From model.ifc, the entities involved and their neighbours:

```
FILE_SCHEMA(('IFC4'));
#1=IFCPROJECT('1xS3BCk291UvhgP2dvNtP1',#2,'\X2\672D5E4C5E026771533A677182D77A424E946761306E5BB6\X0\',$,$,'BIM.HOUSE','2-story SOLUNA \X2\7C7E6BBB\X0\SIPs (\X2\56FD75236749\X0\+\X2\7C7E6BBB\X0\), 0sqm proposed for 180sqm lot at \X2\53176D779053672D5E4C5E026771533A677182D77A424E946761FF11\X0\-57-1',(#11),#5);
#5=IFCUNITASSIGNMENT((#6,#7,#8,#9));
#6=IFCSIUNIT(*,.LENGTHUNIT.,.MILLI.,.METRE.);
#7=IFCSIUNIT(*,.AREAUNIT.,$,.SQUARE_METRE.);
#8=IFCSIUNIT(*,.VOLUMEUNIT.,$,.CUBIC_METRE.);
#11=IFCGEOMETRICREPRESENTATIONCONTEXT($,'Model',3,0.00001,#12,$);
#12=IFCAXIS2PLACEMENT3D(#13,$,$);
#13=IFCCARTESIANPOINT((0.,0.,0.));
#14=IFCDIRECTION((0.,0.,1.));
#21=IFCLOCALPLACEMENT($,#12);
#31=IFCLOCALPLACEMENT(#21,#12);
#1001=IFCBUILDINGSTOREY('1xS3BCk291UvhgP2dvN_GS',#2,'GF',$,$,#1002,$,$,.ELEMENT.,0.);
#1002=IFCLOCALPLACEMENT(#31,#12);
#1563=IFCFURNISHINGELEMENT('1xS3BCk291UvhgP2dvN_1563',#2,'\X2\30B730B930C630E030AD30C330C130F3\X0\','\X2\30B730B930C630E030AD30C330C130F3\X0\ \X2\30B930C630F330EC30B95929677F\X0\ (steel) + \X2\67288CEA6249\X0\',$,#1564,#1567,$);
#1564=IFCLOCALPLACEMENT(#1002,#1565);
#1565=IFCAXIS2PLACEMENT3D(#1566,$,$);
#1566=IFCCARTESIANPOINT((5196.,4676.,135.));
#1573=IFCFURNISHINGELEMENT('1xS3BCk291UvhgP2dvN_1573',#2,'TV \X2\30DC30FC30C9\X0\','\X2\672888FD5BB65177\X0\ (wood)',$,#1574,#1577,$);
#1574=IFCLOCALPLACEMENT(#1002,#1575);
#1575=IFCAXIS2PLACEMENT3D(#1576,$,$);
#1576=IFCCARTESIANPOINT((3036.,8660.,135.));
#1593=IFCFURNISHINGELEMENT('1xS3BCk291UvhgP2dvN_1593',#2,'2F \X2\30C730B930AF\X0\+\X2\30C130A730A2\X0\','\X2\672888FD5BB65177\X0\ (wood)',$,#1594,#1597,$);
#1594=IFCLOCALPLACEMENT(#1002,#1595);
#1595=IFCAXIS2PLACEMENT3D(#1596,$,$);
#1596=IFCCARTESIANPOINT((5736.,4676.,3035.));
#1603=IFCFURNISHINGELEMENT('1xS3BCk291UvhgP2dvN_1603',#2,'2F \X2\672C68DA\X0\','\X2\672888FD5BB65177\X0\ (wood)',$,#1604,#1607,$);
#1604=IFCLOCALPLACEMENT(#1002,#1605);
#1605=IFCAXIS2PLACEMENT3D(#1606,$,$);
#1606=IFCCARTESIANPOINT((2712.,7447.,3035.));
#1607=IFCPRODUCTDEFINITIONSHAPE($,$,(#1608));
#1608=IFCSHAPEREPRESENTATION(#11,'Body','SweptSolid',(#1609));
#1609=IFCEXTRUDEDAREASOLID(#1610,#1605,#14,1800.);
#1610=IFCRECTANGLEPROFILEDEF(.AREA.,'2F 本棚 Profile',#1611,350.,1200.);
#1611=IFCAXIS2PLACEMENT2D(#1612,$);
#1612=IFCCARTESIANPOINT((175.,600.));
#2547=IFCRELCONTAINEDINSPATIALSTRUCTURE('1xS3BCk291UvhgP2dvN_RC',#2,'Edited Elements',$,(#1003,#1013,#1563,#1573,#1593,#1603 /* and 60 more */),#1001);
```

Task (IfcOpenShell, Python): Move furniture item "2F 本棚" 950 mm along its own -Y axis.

```python
import ifcopenshell
import ifcopenshell.api.geometry
import ifcopenshell.util.placement

model = ifcopenshell.open("model.ifc")

item = model.by_guid("1xS3BCk291UvhgP2dvN_1603")
matrix = ifcopenshell.util.placement.get_local_placement(item.ObjectPlacement)
matrix[:3, 3] -= matrix[:3, 1] * 950.0
ifcopenshell.api.geometry.edit_object_placement(model, product=item, matrix=matrix, is_si=False)

print(ifcopenshell.util.placement.get_local_placement(item.ObjectPlacement).round(3) + 0.0)

model.write("model-out.ifc")
```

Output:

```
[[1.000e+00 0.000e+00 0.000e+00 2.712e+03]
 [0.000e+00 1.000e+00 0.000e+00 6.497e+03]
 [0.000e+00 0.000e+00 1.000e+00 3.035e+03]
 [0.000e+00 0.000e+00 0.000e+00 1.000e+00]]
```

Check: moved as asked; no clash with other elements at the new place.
